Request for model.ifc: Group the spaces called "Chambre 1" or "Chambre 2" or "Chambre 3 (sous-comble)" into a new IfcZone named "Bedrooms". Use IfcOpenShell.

First a look at what the model holds.

```python
import ifcopenshell

model = ifcopenshell.open("model.ifc")
print(model.schema)
seen = {}
for space in model.by_type("IfcSpace"):
    seen[space.LongName] = seen.get(space.LongName, 0) + 1
for name, count in sorted(seen.items(), key=str):
    print(count, "x", name)
print("zones:", [z.Name for z in model.by_type("IfcZone")][:20])
```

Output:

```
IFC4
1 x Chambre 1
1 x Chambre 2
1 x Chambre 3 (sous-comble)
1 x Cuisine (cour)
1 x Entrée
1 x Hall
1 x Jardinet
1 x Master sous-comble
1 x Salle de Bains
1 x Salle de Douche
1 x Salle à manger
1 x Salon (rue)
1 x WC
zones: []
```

```python
import ifcopenshell
import ifcopenshell.api.group
import ifcopenshell.api.root

model = ifcopenshell.open("model.ifc")

names = {"Chambre 1", "Chambre 2", "Chambre 3 (sous-comble)"}
spaces = [s for s in model.by_type("IfcSpace") if s.LongName in names]

zone = ifcopenshell.api.root.create_entity(model, ifc_class="IfcZone", name="Bedrooms")
ifcopenshell.api.group.assign_group(model, products=spaces, group=zone)
print(len(spaces), "spaces in", zone.Name)

model.write("model_edited.ifc")
```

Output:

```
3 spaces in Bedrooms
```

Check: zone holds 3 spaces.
